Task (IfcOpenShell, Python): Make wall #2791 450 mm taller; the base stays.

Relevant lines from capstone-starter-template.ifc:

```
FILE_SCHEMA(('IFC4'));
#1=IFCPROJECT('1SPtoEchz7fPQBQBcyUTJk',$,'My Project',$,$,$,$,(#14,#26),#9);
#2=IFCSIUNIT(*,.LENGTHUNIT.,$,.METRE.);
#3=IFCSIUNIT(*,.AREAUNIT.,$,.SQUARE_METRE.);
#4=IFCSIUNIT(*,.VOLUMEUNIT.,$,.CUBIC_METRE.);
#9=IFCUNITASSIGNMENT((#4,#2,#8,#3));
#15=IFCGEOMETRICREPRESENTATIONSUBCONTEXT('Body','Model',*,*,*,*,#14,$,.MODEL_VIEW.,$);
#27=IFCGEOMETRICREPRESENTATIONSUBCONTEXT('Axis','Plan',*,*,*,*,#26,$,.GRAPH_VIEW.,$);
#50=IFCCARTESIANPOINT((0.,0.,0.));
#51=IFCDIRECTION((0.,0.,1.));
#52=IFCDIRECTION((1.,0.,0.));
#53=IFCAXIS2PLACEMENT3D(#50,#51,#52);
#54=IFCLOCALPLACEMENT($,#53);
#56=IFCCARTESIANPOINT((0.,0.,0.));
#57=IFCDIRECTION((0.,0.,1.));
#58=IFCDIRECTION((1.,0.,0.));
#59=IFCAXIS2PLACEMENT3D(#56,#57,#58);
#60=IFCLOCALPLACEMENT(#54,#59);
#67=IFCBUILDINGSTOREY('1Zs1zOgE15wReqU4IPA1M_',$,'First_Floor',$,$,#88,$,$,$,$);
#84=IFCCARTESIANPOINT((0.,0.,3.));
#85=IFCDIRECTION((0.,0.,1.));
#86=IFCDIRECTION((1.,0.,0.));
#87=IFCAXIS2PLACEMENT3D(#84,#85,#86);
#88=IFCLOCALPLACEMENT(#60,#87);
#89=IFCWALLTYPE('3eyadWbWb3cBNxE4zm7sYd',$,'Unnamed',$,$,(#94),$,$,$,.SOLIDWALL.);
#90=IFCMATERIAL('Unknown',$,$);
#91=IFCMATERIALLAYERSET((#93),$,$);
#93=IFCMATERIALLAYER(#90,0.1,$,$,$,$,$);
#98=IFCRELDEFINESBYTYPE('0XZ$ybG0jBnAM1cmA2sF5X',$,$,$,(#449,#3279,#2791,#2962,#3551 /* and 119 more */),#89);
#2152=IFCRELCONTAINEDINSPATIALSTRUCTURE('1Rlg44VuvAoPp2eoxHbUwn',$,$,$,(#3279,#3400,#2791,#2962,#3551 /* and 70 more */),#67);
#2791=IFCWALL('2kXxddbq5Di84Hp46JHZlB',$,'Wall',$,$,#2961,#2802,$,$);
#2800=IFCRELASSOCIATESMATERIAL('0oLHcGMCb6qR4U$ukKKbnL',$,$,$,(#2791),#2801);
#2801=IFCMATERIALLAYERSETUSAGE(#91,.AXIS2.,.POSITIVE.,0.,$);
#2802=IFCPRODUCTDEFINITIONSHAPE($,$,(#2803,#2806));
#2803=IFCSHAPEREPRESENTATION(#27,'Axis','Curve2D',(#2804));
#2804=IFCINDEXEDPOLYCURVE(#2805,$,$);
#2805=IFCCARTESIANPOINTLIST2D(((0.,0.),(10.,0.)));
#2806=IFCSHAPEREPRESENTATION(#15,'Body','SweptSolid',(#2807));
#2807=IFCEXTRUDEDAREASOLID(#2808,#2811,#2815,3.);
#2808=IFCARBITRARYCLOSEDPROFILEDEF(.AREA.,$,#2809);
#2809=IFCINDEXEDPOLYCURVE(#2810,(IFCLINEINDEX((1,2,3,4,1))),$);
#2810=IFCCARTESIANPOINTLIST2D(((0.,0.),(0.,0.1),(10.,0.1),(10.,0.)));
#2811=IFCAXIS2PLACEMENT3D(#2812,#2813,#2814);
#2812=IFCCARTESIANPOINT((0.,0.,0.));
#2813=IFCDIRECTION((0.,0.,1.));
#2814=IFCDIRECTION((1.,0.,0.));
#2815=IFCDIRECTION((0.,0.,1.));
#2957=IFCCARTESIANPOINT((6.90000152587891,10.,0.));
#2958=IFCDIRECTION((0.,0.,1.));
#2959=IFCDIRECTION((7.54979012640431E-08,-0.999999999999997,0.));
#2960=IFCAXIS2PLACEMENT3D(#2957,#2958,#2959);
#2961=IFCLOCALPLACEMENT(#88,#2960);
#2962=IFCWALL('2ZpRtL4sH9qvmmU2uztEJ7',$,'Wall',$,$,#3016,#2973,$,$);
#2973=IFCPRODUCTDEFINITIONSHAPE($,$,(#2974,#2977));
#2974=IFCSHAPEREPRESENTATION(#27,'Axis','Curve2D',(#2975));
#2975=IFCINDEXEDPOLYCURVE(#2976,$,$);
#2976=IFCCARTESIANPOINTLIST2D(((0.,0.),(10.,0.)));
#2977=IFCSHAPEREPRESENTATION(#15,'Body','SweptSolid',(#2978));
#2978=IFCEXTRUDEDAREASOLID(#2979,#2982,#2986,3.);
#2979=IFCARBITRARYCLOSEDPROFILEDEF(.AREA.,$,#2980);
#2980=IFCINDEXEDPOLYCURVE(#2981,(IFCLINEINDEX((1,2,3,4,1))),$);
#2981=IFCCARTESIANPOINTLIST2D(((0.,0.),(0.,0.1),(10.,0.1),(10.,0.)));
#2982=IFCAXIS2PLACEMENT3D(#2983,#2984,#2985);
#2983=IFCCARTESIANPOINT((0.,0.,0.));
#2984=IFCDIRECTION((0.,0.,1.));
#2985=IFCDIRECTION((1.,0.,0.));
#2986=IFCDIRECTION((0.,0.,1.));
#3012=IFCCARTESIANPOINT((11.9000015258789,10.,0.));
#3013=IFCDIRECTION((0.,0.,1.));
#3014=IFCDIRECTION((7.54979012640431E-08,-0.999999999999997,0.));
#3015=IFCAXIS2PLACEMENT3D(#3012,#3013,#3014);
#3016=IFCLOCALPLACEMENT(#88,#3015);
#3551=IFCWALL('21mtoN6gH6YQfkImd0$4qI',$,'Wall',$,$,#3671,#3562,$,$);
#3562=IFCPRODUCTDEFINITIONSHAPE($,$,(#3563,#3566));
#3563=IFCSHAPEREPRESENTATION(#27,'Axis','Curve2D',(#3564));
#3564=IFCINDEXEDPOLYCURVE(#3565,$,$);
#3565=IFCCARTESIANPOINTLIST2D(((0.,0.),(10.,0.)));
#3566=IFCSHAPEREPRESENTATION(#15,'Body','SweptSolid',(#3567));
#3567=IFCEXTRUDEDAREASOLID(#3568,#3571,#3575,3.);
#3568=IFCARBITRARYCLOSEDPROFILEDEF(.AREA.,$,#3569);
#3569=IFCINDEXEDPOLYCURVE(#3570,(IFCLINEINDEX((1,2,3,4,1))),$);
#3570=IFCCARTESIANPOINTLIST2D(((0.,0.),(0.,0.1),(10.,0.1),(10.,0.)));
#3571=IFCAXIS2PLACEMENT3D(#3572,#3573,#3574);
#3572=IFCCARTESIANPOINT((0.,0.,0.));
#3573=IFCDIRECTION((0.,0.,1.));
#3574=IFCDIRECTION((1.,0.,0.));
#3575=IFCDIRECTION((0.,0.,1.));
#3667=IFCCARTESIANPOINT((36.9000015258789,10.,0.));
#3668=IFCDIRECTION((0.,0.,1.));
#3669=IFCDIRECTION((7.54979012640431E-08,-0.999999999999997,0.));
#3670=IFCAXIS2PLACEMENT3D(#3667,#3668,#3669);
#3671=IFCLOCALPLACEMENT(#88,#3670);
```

```python
import ifcopenshell
import ifcopenshell.geom
import ifcopenshell.util.representation
import ifcopenshell.util.shape
import ifcopenshell.util.unit

model = ifcopenshell.open("capstone-starter-template.ifc")
unit_scale = ifcopenshell.util.unit.calculate_unit_scale(model)
settings = ifcopenshell.geom.settings()


def volume(element):
    """Net volume in cubic metres, openings subtracted."""
    shape = ifcopenshell.geom.create_shape(settings, element)
    return ifcopenshell.util.shape.get_volume(shape.geometry)


wall = model.by_guid("2kXxddbq5Di84Hp46JHZlB")
before = volume(wall)

body = ifcopenshell.util.representation.get_representation(wall, "Model", "Body")
solid = body.Items[0]
old_height = solid.Depth
solid.Depth += 0.45 / unit_scale
after = volume(wall)

print(f"height {old_height:g} -> {solid.Depth:g}, volume {before:.3f} -> {after:.3f} m3")

model.write("capstone-starter-template_edited.ifc")
```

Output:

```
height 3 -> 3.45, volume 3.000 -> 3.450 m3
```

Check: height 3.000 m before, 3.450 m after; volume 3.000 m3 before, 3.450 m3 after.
